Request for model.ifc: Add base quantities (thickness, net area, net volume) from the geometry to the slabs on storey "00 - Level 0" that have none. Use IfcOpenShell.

First a look at what the model holds.

```python
import ifcopenshell
import ifcopenshell.util.element
import ifcopenshell.util.unit

model = ifcopenshell.open("model.ifc")
print(model.schema)
for unit_type in ("LENGTHUNIT", "AREAUNIT", "VOLUMEUNIT"):
    print(unit_type, ifcopenshell.util.unit.calculate_unit_scale(model, unit_type))
storey = next(s for s in model.by_type("IfcBuildingStorey") if s.Name == "00 - Level 0")
slabs = [e for e in ifcopenshell.util.element.get_decomposition(storey) if e.is_a("IfcSlab")]
for e in sorted(slabs, key=lambda e: e.id()):
    print(e.id(), e.is_a(), e.Name, list(ifcopenshell.util.element.get_psets(e, qtos_only=True)), sep=" | ")
```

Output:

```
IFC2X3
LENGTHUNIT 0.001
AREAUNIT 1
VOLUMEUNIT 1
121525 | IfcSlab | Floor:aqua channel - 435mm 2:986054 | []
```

```python
import ifcopenshell
import ifcopenshell.api.pset
import ifcopenshell.geom
import ifcopenshell.util.element
import ifcopenshell.util.shape
import ifcopenshell.util.unit

model = ifcopenshell.open("model.ifc")
unit_scale = ifcopenshell.util.unit.calculate_unit_scale(model)
area_scale = ifcopenshell.util.unit.calculate_unit_scale(model, "AREAUNIT")
volume_scale = ifcopenshell.util.unit.calculate_unit_scale(model, "VOLUMEUNIT")
settings = ifcopenshell.geom.settings()

storey = next(s for s in model.by_type("IfcBuildingStorey") if s.Name == "00 - Level 0")
slabs = [e for e in ifcopenshell.util.element.get_decomposition(storey) if e.is_a("IfcSlab")]

for e in sorted(slabs, key=lambda e: e.id()):
    if ifcopenshell.util.element.get_psets(e, qtos_only=True, should_inherit=False):
        continue
    # Geometry comes back in metres, in the element's own axes.
    shape = ifcopenshell.geom.create_shape(settings, e)
    values = {
        "Width": ifcopenshell.util.shape.get_z(shape.geometry) / unit_scale,
        "NetArea": ifcopenshell.util.shape.get_footprint_area(shape.geometry) / area_scale,
        "NetVolume": ifcopenshell.util.shape.get_volume(shape.geometry) / volume_scale,
    }
    qto = ifcopenshell.api.pset.add_qto(model, product=e, name="BaseQuantities")
    ifcopenshell.api.pset.edit_qto(model, qto=qto, properties=values)
    print(e.id(), {k: round(v, 3) for k, v in values.items()})

model.write("model_updated.ifc")
```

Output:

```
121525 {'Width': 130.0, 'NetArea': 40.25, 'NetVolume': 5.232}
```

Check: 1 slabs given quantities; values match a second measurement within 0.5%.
